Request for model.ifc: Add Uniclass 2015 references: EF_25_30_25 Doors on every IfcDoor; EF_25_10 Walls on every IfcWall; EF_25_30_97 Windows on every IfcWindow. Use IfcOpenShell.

First a look at what the model holds.

```python
import ifcopenshell

model = ifcopenshell.open("model.ifc")
print(model.schema)
print("classifications:", [c.Name for c in model.by_type("IfcClassification")])
for ifc_class in ("IfcDoor", "IfcRoof", "IfcStair", "IfcWall", "IfcWindow"):
    print(ifc_class, len(model.by_type(ifc_class)))
```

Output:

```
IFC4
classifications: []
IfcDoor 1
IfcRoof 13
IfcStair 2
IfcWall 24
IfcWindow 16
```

```python
import ifcopenshell
import ifcopenshell.api.classification

model = ifcopenshell.open("model.ifc")

system = ifcopenshell.api.classification.add_classification(model, classification="Uniclass 2015")

codes = {
    "IfcDoor": ("EF_25_30_25", "Doors"),
    "IfcWall": ("EF_25_10", "Walls"),
    "IfcWindow": ("EF_25_30_97", "Windows"),
}
for ifc_class, (code, name) in codes.items():
    products = model.by_type(ifc_class)
    ifcopenshell.api.classification.add_reference(
        model, products=products, classification=system, identification=code, name=name
    )
    print(code, len(products))

model.write("model_edited.ifc")
```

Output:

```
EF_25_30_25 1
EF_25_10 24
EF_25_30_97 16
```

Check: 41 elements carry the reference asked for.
